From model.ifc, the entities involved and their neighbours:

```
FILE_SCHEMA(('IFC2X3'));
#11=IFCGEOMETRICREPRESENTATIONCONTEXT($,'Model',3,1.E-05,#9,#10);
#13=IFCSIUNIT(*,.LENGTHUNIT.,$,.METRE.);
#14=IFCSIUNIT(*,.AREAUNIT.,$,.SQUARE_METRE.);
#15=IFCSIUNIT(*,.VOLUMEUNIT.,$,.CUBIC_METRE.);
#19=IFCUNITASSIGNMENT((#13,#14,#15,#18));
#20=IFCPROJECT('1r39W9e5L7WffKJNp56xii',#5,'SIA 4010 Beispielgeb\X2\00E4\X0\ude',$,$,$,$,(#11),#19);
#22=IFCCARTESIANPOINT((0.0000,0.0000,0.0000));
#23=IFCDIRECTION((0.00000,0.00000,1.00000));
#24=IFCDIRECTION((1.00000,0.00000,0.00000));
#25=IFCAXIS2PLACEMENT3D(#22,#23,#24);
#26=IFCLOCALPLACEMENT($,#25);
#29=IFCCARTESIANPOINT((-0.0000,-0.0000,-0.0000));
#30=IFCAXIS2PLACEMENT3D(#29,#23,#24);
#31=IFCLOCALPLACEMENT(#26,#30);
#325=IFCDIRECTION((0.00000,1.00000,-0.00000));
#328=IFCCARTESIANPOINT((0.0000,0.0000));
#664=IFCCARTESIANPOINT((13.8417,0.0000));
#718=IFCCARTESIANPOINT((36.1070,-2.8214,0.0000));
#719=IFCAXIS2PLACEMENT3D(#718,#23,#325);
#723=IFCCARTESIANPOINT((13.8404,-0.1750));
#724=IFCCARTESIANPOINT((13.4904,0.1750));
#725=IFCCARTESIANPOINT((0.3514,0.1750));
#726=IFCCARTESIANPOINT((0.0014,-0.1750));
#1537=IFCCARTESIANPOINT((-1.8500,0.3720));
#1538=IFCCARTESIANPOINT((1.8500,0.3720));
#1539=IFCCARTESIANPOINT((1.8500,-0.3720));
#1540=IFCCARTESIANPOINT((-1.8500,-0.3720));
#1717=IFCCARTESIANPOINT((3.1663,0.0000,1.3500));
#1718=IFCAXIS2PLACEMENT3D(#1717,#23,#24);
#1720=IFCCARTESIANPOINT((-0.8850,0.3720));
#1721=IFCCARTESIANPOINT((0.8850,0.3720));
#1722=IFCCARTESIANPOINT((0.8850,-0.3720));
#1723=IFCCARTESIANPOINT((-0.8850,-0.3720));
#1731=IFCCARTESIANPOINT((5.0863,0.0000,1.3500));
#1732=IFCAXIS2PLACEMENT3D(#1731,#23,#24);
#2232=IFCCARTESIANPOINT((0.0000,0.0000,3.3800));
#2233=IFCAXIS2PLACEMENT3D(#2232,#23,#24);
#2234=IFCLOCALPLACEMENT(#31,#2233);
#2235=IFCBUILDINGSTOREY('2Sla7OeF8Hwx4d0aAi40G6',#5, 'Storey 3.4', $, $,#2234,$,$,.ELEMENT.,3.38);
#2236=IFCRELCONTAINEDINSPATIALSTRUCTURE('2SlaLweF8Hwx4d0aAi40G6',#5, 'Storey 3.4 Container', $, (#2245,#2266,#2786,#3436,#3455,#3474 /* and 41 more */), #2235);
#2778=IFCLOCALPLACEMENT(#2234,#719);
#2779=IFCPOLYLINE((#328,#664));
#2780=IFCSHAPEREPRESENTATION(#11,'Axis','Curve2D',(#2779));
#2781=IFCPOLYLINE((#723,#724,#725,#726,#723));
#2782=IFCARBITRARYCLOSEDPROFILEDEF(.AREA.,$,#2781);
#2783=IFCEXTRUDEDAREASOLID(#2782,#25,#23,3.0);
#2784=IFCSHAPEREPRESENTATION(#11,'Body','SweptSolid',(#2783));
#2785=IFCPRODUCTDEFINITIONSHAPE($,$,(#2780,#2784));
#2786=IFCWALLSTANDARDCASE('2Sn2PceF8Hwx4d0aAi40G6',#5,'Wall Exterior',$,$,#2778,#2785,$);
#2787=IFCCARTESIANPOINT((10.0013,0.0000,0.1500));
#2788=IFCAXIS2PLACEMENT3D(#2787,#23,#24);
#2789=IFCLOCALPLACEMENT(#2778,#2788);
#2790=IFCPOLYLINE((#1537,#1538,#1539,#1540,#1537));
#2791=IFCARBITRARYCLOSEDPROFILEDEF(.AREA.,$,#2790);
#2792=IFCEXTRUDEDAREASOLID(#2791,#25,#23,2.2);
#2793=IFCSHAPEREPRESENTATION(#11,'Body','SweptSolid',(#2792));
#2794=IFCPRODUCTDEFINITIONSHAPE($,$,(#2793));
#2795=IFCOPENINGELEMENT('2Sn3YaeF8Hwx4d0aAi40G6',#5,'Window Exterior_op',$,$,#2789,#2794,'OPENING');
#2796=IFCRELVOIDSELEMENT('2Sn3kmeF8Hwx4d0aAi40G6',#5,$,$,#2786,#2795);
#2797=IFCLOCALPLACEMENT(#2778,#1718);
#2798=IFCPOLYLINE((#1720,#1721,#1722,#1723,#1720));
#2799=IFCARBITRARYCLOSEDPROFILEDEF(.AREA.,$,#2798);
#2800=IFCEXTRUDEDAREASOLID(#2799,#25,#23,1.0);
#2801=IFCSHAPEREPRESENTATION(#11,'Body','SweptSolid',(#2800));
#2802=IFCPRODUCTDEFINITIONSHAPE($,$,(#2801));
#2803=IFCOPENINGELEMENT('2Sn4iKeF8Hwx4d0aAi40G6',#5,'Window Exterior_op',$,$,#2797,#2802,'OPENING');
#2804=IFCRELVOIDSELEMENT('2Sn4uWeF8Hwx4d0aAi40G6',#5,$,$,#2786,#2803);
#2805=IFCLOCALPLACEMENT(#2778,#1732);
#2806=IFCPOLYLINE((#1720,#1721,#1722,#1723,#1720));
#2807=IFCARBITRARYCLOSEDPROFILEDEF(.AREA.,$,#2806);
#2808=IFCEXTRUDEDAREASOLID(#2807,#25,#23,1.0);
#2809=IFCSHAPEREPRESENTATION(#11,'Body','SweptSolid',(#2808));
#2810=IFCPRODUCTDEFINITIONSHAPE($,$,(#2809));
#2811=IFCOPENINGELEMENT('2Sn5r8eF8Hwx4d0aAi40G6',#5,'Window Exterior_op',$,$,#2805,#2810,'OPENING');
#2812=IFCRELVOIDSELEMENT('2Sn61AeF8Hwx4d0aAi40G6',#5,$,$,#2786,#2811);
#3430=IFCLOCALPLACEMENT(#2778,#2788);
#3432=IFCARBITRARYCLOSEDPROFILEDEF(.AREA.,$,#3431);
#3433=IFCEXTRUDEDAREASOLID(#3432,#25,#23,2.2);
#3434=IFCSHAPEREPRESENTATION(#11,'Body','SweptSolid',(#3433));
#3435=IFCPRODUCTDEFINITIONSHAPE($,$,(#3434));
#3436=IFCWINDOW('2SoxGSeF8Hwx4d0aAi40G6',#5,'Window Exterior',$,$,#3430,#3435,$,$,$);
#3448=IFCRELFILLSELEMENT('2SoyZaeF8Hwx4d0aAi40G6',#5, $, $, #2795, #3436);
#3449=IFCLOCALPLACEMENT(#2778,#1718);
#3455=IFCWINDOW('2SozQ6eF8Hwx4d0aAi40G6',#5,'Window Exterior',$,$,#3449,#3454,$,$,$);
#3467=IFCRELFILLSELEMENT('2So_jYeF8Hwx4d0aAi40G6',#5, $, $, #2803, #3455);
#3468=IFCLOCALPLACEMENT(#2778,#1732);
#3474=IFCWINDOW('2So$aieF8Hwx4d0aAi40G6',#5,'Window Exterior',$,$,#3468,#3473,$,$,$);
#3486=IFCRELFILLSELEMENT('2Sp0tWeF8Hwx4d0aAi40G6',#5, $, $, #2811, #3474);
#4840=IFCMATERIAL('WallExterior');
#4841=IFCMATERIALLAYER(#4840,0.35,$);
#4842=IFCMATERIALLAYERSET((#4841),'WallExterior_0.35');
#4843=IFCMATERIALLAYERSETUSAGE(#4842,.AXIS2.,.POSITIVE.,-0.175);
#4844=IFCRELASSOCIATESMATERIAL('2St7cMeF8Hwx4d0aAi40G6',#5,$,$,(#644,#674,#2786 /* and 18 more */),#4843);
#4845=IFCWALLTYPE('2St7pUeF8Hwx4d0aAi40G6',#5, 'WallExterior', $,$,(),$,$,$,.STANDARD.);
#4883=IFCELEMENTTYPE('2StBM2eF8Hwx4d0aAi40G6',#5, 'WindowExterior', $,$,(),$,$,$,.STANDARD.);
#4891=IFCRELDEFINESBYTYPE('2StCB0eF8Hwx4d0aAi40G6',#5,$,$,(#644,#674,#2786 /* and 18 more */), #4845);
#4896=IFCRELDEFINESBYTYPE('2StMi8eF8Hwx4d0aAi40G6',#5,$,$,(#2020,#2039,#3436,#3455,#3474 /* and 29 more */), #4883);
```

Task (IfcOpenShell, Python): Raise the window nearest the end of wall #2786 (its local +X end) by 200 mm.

```python
import numpy as np
import ifcopenshell
import ifcopenshell.api.geometry
import ifcopenshell.util.placement
import ifcopenshell.util.unit

model = ifcopenshell.open("model.ifc")
unit_scale = ifcopenshell.util.unit.calculate_unit_scale(model)

window = model.by_guid("2SoxGSeF8Hwx4d0aAi40G6")
opening = window.FillsVoids[0].RelatingOpeningElement
dz = 0.2 / unit_scale

shift = np.array([0.0, 0.0, dz])
# The window is not placed relative to its opening, so move both.
for product in (opening, window):
    matrix = ifcopenshell.util.placement.get_local_placement(product.ObjectPlacement)
    matrix[:3, 3] += shift
    ifcopenshell.api.geometry.edit_object_placement(model, product=product, matrix=matrix, is_si=False)

print(f"moved by {dz * unit_scale:+.3f} m")

model.write("model_updated.ifc")
```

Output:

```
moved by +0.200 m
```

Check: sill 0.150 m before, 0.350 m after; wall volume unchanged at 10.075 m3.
